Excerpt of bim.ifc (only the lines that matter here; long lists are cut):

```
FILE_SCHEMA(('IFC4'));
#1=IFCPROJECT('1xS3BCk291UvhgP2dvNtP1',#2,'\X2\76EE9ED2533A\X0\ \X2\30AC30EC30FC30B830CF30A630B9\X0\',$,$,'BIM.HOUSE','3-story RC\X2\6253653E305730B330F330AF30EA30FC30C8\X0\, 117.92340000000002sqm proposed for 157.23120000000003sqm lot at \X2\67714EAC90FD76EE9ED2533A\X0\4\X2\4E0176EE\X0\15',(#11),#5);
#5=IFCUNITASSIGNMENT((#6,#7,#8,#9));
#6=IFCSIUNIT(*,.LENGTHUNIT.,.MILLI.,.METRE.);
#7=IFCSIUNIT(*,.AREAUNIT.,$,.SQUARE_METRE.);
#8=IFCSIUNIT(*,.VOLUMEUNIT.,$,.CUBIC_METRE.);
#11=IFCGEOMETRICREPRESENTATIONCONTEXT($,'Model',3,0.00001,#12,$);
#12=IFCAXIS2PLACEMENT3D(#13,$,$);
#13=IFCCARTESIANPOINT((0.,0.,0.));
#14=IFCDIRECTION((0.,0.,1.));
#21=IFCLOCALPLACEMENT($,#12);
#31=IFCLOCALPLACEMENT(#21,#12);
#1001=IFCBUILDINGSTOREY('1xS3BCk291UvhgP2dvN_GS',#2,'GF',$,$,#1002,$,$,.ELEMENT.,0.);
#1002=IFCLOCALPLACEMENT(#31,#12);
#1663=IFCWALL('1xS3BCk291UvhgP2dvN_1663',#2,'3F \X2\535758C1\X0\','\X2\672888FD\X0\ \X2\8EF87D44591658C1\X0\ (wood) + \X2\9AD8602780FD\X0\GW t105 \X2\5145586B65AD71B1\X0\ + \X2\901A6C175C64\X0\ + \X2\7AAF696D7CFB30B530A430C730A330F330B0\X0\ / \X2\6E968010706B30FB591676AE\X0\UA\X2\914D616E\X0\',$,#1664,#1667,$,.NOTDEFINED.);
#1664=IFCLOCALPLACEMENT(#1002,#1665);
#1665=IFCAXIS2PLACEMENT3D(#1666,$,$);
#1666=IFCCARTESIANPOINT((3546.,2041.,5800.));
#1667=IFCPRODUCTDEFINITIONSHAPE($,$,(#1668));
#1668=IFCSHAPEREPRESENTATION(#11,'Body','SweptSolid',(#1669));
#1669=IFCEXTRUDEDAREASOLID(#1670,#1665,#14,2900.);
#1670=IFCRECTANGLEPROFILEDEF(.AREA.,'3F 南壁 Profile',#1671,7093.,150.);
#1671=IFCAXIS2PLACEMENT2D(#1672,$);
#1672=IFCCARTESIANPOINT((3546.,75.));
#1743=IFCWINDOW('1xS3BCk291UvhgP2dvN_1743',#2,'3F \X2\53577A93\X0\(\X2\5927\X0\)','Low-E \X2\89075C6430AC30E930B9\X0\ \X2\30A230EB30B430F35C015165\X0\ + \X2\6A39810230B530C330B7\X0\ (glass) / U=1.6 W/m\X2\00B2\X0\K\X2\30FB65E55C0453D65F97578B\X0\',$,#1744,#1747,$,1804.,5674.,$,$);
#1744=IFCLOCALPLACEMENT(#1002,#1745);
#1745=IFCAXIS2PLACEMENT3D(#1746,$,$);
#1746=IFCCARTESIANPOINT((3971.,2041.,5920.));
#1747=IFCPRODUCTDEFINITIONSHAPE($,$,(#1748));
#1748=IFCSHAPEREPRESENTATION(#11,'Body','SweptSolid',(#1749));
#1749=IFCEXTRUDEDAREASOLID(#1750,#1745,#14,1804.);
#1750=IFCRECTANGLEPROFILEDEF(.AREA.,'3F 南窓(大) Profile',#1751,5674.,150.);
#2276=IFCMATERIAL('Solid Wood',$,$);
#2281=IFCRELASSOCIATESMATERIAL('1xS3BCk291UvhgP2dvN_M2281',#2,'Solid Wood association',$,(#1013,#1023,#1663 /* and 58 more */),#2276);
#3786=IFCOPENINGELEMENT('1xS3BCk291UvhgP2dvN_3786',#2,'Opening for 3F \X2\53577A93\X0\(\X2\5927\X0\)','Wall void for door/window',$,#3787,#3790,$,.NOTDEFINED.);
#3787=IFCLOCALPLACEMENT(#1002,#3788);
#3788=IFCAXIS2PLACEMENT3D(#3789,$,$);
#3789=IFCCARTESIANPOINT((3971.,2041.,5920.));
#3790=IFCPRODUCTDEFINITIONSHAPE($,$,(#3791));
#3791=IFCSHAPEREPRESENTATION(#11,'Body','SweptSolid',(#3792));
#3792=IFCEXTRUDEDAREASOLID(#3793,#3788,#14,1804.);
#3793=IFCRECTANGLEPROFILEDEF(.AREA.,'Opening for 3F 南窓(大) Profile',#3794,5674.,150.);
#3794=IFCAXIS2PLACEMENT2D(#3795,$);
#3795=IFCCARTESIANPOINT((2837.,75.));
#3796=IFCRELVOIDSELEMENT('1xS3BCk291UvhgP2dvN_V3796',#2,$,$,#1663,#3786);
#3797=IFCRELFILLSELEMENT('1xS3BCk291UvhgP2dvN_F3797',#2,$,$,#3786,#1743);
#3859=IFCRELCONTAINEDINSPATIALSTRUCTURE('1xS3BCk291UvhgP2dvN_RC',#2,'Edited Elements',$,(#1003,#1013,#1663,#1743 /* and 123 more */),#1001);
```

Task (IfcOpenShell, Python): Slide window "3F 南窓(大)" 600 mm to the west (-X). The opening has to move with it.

```python
import ifcopenshell
import ifcopenshell.api.geometry
import ifcopenshell.util.placement

model = ifcopenshell.open("bim.ifc")

window = model.by_guid("1xS3BCk291UvhgP2dvN_1743")
opening = window.FillsVoids[0].RelatingOpeningElement
wall = opening.VoidsElements[0].RelatingBuildingElement

wall_matrix = ifcopenshell.util.placement.get_local_placement(wall.ObjectPlacement)
shift = wall_matrix[:3, 0] * -600.0
before = ifcopenshell.util.placement.get_local_placement(window.ObjectPlacement)[:3, 3].copy()

# The window is not placed relative to its opening, so move both.
for product in (opening, window):
    matrix = ifcopenshell.util.placement.get_local_placement(product.ObjectPlacement)
    matrix[:3, 3] += shift
    ifcopenshell.api.geometry.edit_object_placement(model, product=product, matrix=matrix, is_si=False)

after = ifcopenshell.util.placement.get_local_placement(window.ObjectPlacement)[:3, 3]
print("window moved by", (after - before).round(3) + 0.0)

model.write("bim_edited.ifc")
```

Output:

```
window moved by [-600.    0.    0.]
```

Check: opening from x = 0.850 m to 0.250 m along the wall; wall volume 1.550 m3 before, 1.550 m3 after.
